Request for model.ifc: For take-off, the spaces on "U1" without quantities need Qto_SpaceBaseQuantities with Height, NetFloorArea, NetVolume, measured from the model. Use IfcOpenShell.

First a look at what the model holds.

```python
import ifcopenshell
import ifcopenshell.util.element
import ifcopenshell.util.unit

model = ifcopenshell.open("model.ifc")
print(model.schema)
for unit_type in ("LENGTHUNIT", "AREAUNIT", "VOLUMEUNIT"):
    print(unit_type, ifcopenshell.util.unit.calculate_unit_scale(model, unit_type))
storey = next(s for s in model.by_type("IfcBuildingStorey") if s.Name == "U1")
spaces = [e for e in ifcopenshell.util.element.get_decomposition(storey) if e.is_a("IfcSpace")]
for e in sorted(spaces, key=lambda e: e.id()):
    print(e.id(), e.is_a(), e.Name, list(ifcopenshell.util.element.get_psets(e, qtos_only=True)), sep=" | ")
```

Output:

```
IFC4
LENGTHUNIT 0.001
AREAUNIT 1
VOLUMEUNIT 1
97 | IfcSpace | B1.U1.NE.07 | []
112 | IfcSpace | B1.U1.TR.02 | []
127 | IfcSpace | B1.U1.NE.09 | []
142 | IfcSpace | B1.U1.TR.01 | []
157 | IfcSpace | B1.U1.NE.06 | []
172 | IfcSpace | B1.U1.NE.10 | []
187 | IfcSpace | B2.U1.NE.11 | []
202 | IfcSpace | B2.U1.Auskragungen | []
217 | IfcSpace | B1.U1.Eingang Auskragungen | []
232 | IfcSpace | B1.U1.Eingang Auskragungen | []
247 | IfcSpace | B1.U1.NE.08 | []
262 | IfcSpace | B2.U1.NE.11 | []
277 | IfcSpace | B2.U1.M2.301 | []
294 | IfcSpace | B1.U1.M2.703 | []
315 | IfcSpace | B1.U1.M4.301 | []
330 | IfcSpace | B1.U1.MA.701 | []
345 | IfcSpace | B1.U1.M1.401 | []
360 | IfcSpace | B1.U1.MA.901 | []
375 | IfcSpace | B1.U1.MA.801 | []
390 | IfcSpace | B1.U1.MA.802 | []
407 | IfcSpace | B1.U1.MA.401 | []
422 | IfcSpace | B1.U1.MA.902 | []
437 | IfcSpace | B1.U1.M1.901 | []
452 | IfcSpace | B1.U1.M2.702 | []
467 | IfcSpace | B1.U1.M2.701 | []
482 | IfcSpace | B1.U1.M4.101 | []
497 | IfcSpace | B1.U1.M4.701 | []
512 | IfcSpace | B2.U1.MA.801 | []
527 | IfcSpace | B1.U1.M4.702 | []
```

```python
import ifcopenshell
import ifcopenshell.api.pset
import ifcopenshell.geom
import ifcopenshell.util.element
import ifcopenshell.util.shape
import ifcopenshell.util.unit

model = ifcopenshell.open("model.ifc")
unit_scale = ifcopenshell.util.unit.calculate_unit_scale(model)
area_scale = ifcopenshell.util.unit.calculate_unit_scale(model, "AREAUNIT")
volume_scale = ifcopenshell.util.unit.calculate_unit_scale(model, "VOLUMEUNIT")
settings = ifcopenshell.geom.settings()

storey = next(s for s in model.by_type("IfcBuildingStorey") if s.Name == "U1")
spaces = [e for e in ifcopenshell.util.element.get_decomposition(storey) if e.is_a("IfcSpace")]

for e in sorted(spaces, key=lambda e: e.id()):
    if ifcopenshell.util.element.get_psets(e, qtos_only=True, should_inherit=False):
        continue
    # Geometry comes back in metres, in the element's own axes.
    shape = ifcopenshell.geom.create_shape(settings, e)
    values = {
        "Height": ifcopenshell.util.shape.get_z(shape.geometry) / unit_scale,
        "NetFloorArea": ifcopenshell.util.shape.get_footprint_area(shape.geometry) / area_scale,
        "NetVolume": ifcopenshell.util.shape.get_volume(shape.geometry) / volume_scale,
    }
    qto = ifcopenshell.api.pset.add_qto(model, product=e, name="Qto_SpaceBaseQuantities")
    ifcopenshell.api.pset.edit_qto(model, qto=qto, properties=values)
    print(e.id(), {k: round(v, 3) for k, v in values.items()})

model.write("model_edited.ifc")
```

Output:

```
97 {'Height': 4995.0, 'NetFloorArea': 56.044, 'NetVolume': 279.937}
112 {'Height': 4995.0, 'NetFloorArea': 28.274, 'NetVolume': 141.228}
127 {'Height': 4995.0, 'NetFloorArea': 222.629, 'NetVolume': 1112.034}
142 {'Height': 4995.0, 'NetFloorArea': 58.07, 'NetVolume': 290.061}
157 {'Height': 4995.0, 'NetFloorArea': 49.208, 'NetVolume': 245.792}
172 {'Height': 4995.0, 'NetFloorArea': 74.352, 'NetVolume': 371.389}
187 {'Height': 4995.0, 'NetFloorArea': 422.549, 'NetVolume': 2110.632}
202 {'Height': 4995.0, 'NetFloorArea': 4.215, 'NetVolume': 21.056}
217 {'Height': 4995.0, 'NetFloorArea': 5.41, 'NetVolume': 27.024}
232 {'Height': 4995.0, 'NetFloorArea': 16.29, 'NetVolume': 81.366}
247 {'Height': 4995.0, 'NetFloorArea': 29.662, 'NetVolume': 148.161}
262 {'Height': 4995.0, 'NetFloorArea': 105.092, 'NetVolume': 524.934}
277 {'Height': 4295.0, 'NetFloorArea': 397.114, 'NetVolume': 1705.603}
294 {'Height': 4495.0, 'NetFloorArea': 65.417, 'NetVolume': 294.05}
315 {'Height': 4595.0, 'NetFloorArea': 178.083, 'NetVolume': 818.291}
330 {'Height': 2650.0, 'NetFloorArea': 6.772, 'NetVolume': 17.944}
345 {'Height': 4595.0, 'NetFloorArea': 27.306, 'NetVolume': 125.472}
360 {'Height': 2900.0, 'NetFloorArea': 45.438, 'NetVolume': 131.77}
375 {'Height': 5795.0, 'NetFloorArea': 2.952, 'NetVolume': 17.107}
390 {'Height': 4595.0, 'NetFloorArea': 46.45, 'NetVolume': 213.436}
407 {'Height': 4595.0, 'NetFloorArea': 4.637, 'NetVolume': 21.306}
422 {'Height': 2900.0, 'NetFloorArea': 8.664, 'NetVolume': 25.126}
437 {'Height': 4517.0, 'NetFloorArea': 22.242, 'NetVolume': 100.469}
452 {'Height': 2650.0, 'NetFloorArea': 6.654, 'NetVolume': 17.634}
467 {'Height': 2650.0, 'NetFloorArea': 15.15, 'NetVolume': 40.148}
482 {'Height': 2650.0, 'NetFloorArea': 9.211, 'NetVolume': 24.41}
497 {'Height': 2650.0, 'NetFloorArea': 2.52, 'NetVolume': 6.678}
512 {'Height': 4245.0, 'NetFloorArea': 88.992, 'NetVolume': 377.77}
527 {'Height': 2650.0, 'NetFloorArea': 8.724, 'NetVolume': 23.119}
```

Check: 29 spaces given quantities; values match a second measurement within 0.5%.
